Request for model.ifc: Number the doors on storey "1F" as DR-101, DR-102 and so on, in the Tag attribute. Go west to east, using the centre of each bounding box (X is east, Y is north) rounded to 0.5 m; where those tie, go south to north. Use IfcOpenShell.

First a look at what the model holds.

```python
import ifcopenshell
import ifcopenshell.util.element
import ifcopenshell.util.placement

model = ifcopenshell.open("model.ifc")
print(model.schema)
storey = next(s for s in model.by_type("IfcBuildingStorey") if s.Name == "1F")
doors = [e for e in ifcopenshell.util.element.get_decomposition(storey) if e.is_a("IfcDoor")]
for e in sorted(doors, key=lambda e: e.id()):
    origin = ifcopenshell.util.placement.get_local_placement(e.ObjectPlacement)[:3, 3]
    print(e.id(), e.Tag, e.Name, origin.round(2) + 0.0, sep=" | ")
```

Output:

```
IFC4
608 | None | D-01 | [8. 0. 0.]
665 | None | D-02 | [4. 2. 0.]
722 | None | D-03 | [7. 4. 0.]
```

```python
import ifcopenshell
import ifcopenshell.geom
import ifcopenshell.util.element
import ifcopenshell.util.shape

model = ifcopenshell.open("model.ifc")
settings = ifcopenshell.geom.settings()
settings.set("use-world-coords", True)


def centre(element):
    shape = ifcopenshell.geom.create_shape(settings, element)
    return ifcopenshell.util.shape.get_bbox_centroid(shape.geometry)


storey = next(s for s in model.by_type("IfcBuildingStorey") if s.Name == "1F")
doors = [e for e in ifcopenshell.util.element.get_decomposition(storey) if e.is_a("IfcDoor")]

# Insertion points can sit at a corner or the storey origin, so sort by the geometry (in metres).
centres = {e: centre(e) for e in doors}
doors.sort(key=lambda e: (round(centres[e][0] / 0.5), centres[e][1]))

for i, e in enumerate(doors, start=1):
    number = f"DR-1{i:02d}"
    e.Tag = number
    print(e.id(), number)

model.write("model-out.ifc")
```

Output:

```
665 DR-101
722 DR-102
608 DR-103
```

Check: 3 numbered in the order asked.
